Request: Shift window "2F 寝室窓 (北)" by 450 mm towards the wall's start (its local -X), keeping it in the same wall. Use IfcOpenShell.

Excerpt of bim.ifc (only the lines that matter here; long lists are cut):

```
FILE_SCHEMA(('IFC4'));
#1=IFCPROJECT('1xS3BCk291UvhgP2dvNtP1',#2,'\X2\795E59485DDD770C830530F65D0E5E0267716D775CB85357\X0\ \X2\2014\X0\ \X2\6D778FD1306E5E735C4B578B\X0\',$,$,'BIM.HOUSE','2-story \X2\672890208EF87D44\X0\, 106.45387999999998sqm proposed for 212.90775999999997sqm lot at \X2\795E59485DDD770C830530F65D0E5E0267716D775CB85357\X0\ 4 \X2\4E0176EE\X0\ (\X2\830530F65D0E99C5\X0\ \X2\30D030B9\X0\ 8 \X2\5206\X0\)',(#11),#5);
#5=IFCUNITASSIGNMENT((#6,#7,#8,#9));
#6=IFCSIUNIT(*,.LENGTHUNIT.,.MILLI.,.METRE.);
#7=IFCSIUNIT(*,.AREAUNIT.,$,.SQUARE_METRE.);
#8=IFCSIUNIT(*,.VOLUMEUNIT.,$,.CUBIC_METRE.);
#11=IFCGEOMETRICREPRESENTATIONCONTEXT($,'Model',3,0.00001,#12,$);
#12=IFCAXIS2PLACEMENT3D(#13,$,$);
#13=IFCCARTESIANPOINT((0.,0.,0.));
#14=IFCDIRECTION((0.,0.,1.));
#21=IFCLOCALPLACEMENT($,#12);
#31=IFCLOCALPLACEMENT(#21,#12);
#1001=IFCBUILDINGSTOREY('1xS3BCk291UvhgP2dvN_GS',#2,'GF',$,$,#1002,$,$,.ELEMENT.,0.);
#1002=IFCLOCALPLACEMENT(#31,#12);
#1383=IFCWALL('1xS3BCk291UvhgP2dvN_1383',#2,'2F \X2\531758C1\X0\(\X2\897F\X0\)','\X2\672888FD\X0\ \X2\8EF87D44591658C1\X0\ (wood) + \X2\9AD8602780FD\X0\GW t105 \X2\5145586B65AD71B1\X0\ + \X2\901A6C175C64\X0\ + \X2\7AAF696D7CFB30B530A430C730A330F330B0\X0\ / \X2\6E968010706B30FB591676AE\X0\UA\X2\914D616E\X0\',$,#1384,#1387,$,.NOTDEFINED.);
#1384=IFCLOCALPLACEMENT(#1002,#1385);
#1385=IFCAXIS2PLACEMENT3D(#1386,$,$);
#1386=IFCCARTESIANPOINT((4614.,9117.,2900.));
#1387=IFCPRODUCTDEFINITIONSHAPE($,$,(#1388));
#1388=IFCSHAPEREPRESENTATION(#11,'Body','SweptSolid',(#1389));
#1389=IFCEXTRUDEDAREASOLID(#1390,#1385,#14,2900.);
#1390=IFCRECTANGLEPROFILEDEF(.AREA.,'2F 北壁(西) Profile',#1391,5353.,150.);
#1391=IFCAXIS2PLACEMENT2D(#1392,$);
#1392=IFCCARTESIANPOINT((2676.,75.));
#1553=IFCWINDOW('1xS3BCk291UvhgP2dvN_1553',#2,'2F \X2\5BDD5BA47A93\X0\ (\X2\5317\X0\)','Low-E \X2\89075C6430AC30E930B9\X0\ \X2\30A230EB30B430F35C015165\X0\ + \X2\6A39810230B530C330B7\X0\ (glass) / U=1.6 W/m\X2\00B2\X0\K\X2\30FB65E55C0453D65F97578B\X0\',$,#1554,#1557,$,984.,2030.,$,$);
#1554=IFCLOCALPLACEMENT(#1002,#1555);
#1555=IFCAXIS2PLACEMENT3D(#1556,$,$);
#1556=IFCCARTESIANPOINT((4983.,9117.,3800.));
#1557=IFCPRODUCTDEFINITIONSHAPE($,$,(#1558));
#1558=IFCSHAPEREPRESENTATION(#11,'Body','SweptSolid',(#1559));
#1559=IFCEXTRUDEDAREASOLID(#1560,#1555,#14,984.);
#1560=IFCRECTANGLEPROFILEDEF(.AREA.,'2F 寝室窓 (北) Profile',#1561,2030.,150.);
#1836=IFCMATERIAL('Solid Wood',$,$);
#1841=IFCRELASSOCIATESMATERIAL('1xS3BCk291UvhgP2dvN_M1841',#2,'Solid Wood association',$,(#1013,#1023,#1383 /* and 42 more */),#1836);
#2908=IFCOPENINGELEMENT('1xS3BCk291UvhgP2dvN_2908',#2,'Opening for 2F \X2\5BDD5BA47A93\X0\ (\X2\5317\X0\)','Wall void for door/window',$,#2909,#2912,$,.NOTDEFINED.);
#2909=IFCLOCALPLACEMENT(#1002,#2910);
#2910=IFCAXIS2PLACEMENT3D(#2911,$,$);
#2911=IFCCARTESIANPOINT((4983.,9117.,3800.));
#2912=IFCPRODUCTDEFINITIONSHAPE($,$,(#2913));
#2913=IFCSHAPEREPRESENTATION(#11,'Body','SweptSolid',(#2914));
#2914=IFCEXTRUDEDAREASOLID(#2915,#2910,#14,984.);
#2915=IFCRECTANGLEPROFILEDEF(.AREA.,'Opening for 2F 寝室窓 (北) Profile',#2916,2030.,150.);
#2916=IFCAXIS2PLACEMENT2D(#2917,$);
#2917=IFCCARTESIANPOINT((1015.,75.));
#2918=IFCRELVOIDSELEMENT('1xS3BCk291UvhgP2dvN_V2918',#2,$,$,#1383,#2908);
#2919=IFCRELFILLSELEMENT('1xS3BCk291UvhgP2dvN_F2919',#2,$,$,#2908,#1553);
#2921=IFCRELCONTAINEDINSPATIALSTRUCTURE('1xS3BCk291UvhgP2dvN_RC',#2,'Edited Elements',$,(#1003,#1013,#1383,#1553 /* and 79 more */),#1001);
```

```python
import ifcopenshell
import ifcopenshell.api.geometry
import ifcopenshell.util.placement

model = ifcopenshell.open("bim.ifc")

window = model.by_id(1553)
opening = window.FillsVoids[0].RelatingOpeningElement
wall = opening.VoidsElements[0].RelatingBuildingElement

wall_matrix = ifcopenshell.util.placement.get_local_placement(wall.ObjectPlacement)
shift = wall_matrix[:3, 0] * -450.0
before = ifcopenshell.util.placement.get_local_placement(window.ObjectPlacement)[:3, 3].copy()

# The window is not placed relative to its opening, so move both.
for product in (opening, window):
    matrix = ifcopenshell.util.placement.get_local_placement(product.ObjectPlacement)
    matrix[:3, 3] += shift
    ifcopenshell.api.geometry.edit_object_placement(model, product=product, matrix=matrix, is_si=False)

after = ifcopenshell.util.placement.get_local_placement(window.ObjectPlacement)[:3, 3]
print("window moved by", (after - before).round(3) + 0.0)

model.write("bim_v2.ifc")
```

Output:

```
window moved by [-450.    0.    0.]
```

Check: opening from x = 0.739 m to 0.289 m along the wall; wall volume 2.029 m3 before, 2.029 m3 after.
